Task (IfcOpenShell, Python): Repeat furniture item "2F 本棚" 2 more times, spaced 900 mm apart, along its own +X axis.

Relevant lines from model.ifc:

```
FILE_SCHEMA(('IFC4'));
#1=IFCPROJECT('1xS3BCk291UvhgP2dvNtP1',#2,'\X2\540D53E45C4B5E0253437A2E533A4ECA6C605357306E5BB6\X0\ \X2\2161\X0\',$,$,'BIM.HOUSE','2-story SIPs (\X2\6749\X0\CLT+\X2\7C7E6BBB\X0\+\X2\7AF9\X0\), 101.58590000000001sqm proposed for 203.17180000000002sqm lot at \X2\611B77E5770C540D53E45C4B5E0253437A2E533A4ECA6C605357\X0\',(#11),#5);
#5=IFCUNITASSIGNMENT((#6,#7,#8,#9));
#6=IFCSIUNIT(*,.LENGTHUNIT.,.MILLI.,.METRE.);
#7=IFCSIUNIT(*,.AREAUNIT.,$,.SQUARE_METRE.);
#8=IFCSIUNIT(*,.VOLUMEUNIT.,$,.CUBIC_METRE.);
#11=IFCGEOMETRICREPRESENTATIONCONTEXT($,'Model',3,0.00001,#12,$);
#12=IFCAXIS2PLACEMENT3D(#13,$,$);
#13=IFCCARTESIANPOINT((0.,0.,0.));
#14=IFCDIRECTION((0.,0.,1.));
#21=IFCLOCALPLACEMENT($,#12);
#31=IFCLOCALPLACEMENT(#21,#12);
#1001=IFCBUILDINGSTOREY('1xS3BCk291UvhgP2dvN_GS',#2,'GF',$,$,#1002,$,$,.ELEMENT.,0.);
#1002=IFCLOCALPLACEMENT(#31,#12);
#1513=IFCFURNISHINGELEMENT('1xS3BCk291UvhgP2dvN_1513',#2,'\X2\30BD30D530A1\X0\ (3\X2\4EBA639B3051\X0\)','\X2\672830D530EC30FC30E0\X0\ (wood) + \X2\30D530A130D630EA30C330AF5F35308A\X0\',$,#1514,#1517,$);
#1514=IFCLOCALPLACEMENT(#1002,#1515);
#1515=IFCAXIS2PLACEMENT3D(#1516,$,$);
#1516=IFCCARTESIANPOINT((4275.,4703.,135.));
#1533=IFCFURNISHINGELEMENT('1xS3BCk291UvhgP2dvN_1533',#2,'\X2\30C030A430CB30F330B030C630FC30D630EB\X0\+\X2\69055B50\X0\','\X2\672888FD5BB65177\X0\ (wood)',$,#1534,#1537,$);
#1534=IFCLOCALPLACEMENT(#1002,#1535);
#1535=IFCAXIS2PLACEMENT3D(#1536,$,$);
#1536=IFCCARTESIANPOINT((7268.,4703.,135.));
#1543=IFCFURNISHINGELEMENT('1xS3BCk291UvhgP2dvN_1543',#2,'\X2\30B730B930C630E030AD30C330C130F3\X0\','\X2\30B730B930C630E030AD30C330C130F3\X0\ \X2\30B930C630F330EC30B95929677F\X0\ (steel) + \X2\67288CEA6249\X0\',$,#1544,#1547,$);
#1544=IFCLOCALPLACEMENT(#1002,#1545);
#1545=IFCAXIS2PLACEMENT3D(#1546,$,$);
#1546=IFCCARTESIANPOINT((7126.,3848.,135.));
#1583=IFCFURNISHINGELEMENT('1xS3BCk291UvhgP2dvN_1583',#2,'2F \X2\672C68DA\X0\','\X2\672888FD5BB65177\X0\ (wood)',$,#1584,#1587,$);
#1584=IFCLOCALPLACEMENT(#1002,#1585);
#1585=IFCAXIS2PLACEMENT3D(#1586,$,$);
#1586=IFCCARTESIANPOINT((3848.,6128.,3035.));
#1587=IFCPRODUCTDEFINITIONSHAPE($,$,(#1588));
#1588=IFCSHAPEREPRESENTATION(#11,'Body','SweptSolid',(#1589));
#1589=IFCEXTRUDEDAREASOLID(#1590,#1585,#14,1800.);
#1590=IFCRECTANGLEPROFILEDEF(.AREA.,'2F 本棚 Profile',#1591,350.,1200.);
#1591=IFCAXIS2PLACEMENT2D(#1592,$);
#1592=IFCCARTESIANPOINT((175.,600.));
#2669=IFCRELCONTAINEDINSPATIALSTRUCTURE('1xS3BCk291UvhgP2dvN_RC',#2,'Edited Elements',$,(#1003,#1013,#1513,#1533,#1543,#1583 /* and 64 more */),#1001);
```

```python
import ifcopenshell
import ifcopenshell.api.geometry
import ifcopenshell.api.root
import ifcopenshell.util.element
import ifcopenshell.util.placement
import ifcopenshell.util.unit

model = ifcopenshell.open("model.ifc")
unit_scale = ifcopenshell.util.unit.calculate_unit_scale(model)


def reuse_history(source, copy):
    """copy_class also copies each property set's owner history, people and application; keep the originals."""
    for rel in copy.IsDefinedBy:
        if rel.is_a("IfcRelDefinesByProperties") and (history := rel.RelatingPropertyDefinition.OwnerHistory):
            rel.RelatingPropertyDefinition.OwnerHistory = source.OwnerHistory
            ifcopenshell.util.element.remove_deep2(model, history)


source = model.by_id(1583)
base = ifcopenshell.util.placement.get_local_placement(source.ObjectPlacement)
step = base[:3, 0] * 0.9 / unit_scale

for i in range(1, 3):
    copy = ifcopenshell.api.root.copy_class(model, product=source)
    copy.Representation = ifcopenshell.util.element.copy_deep(
        model, source.Representation, exclude=["IfcGeometricRepresentationContext", "IfcRepresentationMap"]
    )
    reuse_history(source, copy)
    matrix = base.copy()
    matrix[:3, 3] += i * step
    print("added at", matrix[:3, 3].round(3) + 0.0)
    ifcopenshell.api.geometry.edit_object_placement(model, product=copy, matrix=matrix, is_si=False)

model.write("model_updated.ifc")
```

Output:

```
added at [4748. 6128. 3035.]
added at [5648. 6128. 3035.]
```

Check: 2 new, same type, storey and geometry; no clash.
